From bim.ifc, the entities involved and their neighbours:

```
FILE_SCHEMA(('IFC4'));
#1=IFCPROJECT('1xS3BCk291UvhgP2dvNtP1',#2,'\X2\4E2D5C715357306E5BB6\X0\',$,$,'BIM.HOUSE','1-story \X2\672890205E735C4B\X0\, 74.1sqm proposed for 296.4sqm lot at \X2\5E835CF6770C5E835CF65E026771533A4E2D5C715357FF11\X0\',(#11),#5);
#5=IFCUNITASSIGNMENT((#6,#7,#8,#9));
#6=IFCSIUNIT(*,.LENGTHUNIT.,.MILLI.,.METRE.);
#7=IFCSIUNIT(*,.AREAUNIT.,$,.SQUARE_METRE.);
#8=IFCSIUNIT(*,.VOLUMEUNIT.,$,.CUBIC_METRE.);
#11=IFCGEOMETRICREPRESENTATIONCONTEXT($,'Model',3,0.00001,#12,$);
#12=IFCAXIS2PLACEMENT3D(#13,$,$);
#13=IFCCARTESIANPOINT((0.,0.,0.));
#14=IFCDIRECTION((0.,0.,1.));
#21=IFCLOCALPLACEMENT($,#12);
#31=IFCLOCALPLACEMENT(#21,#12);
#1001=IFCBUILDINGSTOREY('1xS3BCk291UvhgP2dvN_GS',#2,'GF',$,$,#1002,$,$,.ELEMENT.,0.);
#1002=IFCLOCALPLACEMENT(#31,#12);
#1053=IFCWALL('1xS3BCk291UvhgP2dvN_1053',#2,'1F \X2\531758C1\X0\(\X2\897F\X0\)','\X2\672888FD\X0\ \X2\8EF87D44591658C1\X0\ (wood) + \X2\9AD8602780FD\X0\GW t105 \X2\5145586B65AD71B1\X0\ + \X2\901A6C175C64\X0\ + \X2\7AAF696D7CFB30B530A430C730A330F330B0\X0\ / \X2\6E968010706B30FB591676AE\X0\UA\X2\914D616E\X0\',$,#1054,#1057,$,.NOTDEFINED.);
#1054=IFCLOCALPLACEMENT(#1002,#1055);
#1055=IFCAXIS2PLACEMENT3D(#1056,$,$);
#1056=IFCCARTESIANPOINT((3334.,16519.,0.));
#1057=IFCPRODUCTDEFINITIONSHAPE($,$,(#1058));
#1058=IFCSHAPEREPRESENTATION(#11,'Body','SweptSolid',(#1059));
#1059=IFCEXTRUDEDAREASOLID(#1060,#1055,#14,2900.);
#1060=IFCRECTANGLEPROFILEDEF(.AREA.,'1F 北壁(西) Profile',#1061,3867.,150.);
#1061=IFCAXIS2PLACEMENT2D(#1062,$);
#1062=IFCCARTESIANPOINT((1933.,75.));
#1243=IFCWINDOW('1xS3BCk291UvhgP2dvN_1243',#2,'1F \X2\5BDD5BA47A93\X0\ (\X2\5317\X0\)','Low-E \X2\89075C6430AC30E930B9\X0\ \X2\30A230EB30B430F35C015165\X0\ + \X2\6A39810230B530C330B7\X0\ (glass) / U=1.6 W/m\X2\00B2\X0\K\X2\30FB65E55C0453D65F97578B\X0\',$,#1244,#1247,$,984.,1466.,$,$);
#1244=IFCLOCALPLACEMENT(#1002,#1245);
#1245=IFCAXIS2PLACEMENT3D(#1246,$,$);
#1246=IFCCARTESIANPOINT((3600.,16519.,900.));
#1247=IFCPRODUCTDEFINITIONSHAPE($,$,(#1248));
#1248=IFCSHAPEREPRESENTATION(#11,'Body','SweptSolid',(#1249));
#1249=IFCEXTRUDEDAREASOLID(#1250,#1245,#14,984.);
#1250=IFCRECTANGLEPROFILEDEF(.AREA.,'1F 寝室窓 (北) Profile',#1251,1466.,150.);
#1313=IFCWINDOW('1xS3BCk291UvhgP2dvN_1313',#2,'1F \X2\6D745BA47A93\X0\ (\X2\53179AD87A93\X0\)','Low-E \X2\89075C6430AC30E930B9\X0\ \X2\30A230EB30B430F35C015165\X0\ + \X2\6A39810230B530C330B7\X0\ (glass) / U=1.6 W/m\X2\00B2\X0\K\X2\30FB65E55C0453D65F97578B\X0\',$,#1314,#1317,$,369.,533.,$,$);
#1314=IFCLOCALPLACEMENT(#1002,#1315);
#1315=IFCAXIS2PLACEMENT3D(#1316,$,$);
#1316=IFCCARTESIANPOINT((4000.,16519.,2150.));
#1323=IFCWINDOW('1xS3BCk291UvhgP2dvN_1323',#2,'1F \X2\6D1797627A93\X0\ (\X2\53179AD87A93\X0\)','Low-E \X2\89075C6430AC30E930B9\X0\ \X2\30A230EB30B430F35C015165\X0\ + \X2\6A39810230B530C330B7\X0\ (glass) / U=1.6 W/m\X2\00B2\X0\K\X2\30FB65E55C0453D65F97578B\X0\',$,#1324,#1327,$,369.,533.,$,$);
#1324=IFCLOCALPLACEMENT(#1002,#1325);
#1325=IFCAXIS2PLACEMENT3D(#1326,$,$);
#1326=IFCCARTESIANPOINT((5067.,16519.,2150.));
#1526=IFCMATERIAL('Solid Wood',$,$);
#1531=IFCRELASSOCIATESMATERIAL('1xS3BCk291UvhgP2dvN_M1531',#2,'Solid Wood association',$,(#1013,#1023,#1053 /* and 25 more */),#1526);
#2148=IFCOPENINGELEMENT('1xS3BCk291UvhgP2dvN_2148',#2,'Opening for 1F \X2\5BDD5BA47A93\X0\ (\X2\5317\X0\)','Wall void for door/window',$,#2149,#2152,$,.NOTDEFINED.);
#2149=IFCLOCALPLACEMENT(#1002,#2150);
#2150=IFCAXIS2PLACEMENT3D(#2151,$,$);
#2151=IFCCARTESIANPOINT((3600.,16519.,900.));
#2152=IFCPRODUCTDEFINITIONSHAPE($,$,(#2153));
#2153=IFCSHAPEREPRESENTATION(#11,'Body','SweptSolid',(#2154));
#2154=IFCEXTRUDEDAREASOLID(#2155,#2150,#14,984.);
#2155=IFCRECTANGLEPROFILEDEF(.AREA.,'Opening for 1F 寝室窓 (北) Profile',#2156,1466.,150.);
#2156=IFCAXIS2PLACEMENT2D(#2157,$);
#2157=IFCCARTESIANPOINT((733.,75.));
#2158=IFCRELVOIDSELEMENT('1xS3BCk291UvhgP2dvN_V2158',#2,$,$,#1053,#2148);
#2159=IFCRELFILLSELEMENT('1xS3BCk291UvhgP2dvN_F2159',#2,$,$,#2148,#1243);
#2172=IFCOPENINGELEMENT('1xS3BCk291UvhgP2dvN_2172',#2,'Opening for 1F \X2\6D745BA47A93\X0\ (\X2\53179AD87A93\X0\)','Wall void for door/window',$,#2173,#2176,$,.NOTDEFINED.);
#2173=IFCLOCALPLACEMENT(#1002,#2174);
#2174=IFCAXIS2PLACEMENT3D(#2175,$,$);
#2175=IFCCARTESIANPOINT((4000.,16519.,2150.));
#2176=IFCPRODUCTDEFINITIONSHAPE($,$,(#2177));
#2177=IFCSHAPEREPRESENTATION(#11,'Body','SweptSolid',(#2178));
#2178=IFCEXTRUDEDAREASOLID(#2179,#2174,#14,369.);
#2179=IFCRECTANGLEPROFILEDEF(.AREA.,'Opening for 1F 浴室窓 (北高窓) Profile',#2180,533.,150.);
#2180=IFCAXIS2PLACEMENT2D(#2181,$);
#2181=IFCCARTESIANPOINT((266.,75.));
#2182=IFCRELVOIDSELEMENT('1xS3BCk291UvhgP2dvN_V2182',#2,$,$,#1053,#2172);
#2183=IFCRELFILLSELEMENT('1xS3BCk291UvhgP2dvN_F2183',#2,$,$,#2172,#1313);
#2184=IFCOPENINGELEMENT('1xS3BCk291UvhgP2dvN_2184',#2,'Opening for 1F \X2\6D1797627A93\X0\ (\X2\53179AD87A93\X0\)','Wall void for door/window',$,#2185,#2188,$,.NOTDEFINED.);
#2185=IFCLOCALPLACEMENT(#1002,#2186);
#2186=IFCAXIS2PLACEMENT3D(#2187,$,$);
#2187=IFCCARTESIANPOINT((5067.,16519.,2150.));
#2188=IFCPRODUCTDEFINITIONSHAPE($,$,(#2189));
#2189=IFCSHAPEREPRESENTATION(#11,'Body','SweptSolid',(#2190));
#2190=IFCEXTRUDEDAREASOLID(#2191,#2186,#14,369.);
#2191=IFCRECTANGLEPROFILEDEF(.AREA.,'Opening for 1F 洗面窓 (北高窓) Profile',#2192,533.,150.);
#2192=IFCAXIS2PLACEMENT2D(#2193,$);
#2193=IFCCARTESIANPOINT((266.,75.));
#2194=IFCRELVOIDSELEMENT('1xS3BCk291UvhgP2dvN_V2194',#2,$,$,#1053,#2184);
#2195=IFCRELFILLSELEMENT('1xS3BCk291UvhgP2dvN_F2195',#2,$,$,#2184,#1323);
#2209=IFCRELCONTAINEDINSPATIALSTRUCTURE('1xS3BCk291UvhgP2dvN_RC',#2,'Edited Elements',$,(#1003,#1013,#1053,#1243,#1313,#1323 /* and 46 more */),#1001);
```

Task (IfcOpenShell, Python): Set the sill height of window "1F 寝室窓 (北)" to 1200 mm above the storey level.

```python
import numpy as np
import ifcopenshell
import ifcopenshell.api.geometry
import ifcopenshell.geom
import ifcopenshell.util.element
import ifcopenshell.util.placement
import ifcopenshell.util.shape
import ifcopenshell.util.unit

model = ifcopenshell.open("bim.ifc")
unit_scale = ifcopenshell.util.unit.calculate_unit_scale(model)

window = model.by_guid("1xS3BCk291UvhgP2dvN_1243")
opening = window.FillsVoids[0].RelatingOpeningElement
storey = ifcopenshell.util.element.get_container(window, ifc_class="IfcBuildingStorey")
level = ifcopenshell.util.placement.get_local_placement(storey.ObjectPlacement)[2, 3]

# The opening's origin need not be at the sill, so measure its lowest point.
shape = ifcopenshell.geom.create_shape(ifcopenshell.geom.settings(), opening)
bottom = ifcopenshell.util.shape.get_shape_bottom_elevation(shape, shape.geometry) / unit_scale
dz = level + 1.2 / unit_scale - bottom

shift = np.array([0.0, 0.0, dz])
# The window is not placed relative to its opening, so move both.
for product in (opening, window):
    matrix = ifcopenshell.util.placement.get_local_placement(product.ObjectPlacement)
    matrix[:3, 3] += shift
    ifcopenshell.api.geometry.edit_object_placement(model, product=product, matrix=matrix, is_si=False)

print(f"moved by {dz * unit_scale:+.3f} m")

model.write("bim_v2.ifc")
```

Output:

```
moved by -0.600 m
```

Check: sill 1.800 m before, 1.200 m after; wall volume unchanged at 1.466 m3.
